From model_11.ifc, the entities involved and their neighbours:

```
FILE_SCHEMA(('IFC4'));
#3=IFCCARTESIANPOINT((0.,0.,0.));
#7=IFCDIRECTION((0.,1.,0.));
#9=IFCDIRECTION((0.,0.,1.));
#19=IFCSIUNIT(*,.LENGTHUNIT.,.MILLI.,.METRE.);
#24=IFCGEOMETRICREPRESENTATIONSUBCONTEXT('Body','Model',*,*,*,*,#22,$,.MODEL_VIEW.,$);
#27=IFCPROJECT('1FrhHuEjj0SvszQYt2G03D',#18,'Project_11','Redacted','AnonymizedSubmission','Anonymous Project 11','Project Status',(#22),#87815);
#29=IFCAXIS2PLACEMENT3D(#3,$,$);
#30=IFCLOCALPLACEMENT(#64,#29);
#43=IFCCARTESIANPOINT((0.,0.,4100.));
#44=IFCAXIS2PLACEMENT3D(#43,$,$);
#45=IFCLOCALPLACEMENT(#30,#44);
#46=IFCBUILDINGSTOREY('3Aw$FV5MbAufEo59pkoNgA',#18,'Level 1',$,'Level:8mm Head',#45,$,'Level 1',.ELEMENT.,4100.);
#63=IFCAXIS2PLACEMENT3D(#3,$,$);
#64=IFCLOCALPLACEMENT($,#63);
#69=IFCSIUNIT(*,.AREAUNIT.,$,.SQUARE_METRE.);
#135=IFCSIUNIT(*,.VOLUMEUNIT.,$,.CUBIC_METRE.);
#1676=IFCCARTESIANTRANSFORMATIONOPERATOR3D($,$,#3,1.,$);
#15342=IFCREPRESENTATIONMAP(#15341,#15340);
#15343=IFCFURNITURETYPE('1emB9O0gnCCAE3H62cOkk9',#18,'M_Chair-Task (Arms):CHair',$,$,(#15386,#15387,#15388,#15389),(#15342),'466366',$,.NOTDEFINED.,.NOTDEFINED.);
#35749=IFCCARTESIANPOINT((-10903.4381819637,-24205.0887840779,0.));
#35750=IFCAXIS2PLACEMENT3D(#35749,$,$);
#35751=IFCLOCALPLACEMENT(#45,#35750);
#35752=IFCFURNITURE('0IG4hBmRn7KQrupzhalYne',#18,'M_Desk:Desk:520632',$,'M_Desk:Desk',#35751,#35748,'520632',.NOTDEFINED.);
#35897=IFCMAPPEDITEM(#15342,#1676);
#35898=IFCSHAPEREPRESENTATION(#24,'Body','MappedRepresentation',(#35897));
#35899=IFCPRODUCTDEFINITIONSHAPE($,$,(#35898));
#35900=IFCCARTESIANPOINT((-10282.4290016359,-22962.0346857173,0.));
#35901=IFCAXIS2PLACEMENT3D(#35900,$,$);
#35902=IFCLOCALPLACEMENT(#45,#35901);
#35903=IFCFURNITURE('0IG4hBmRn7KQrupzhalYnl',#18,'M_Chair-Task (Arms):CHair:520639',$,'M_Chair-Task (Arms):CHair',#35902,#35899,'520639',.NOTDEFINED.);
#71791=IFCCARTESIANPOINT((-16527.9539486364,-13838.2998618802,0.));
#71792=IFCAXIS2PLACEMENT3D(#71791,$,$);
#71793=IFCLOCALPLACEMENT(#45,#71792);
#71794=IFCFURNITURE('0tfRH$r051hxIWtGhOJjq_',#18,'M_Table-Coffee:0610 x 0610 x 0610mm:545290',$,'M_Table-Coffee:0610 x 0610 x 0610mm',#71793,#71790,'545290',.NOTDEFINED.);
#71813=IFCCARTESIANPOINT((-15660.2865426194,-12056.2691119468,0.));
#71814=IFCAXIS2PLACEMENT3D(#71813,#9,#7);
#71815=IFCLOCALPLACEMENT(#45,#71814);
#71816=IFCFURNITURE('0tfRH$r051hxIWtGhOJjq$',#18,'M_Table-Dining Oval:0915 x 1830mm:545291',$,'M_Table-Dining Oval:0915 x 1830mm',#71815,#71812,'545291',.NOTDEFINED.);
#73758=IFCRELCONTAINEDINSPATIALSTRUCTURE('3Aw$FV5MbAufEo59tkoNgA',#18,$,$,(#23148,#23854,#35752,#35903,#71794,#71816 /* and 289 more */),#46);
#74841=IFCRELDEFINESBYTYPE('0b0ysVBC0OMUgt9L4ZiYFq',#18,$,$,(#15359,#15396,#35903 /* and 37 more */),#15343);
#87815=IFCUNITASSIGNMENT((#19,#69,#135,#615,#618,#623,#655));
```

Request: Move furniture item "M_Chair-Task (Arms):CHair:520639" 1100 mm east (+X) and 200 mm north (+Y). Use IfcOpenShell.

```python
import ifcopenshell
import ifcopenshell.api.geometry
import ifcopenshell.util.placement
import ifcopenshell.util.unit

model = ifcopenshell.open("model_11.ifc")
unit_scale = ifcopenshell.util.unit.calculate_unit_scale(model)

item = model.by_guid("0IG4hBmRn7KQrupzhalYnl")
matrix = ifcopenshell.util.placement.get_local_placement(item.ObjectPlacement)
matrix[0, 3] += 1.1 / unit_scale
matrix[1, 3] += 0.2 / unit_scale
ifcopenshell.api.geometry.edit_object_placement(model, product=item, matrix=matrix, is_si=False)

print(ifcopenshell.util.placement.get_local_placement(item.ObjectPlacement).round(3) + 0.0)

model.write("model_11-out.ifc")
```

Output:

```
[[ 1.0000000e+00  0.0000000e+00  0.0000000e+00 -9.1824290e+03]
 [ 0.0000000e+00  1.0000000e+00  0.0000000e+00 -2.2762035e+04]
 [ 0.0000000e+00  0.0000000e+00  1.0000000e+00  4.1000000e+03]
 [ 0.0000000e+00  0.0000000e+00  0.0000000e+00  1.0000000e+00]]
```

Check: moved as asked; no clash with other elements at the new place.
